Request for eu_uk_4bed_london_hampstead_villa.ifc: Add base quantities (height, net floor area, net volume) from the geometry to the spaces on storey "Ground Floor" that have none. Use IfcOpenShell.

First a look at what the model holds.

```python
import ifcopenshell
import ifcopenshell.util.element
import ifcopenshell.util.unit

model = ifcopenshell.open("eu_uk_4bed_london_hampstead_villa.ifc")
print(model.schema)
for unit_type in ("LENGTHUNIT", "AREAUNIT", "VOLUMEUNIT"):
    print(unit_type, ifcopenshell.util.unit.calculate_unit_scale(model, unit_type))
storey = next(s for s in model.by_type("IfcBuildingStorey") if s.Name == "Ground Floor")
spaces = [e for e in ifcopenshell.util.element.get_decomposition(storey) if e.is_a("IfcSpace")]
for e in sorted(spaces, key=lambda e: e.id()):
    print(e.id(), e.is_a(), e.Name, list(ifcopenshell.util.element.get_psets(e, qtos_only=True)), sep=" | ")
```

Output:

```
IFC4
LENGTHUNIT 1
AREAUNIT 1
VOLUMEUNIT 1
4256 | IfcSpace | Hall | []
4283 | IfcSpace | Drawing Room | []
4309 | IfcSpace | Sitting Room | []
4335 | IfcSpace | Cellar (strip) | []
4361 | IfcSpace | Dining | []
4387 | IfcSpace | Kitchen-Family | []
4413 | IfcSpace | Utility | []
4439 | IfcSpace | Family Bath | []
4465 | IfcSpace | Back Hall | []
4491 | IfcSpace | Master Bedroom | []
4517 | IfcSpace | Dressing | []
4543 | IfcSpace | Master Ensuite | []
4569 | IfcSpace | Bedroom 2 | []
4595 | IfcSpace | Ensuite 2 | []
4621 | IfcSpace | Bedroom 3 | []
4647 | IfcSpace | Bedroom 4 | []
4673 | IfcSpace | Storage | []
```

```python
import ifcopenshell
import ifcopenshell.api.pset
import ifcopenshell.geom
import ifcopenshell.util.element
import ifcopenshell.util.shape
import ifcopenshell.util.unit

model = ifcopenshell.open("eu_uk_4bed_london_hampstead_villa.ifc")
unit_scale = ifcopenshell.util.unit.calculate_unit_scale(model)
area_scale = ifcopenshell.util.unit.calculate_unit_scale(model, "AREAUNIT")
volume_scale = ifcopenshell.util.unit.calculate_unit_scale(model, "VOLUMEUNIT")
settings = ifcopenshell.geom.settings()

storey = next(s for s in model.by_type("IfcBuildingStorey") if s.Name == "Ground Floor")
spaces = [e for e in ifcopenshell.util.element.get_decomposition(storey) if e.is_a("IfcSpace")]

for e in sorted(spaces, key=lambda e: e.id()):
    if ifcopenshell.util.element.get_psets(e, qtos_only=True, should_inherit=False):
        continue
    # Geometry comes back in metres, in the element's own axes.
    shape = ifcopenshell.geom.create_shape(settings, e)
    values = {
        "Height": ifcopenshell.util.shape.get_z(shape.geometry) / unit_scale,
        "NetFloorArea": ifcopenshell.util.shape.get_footprint_area(shape.geometry) / area_scale,
        "NetVolume": ifcopenshell.util.shape.get_volume(shape.geometry) / volume_scale,
    }
    qto = ifcopenshell.api.pset.add_qto(model, product=e, name="Qto_SpaceBaseQuantities")
    ifcopenshell.api.pset.edit_qto(model, qto=qto, properties=values)
    print(e.id(), {k: round(v, 3) for k, v in values.items()})

model.write("eu_uk_4bed_london_hampstead_villa_updated.ifc")
```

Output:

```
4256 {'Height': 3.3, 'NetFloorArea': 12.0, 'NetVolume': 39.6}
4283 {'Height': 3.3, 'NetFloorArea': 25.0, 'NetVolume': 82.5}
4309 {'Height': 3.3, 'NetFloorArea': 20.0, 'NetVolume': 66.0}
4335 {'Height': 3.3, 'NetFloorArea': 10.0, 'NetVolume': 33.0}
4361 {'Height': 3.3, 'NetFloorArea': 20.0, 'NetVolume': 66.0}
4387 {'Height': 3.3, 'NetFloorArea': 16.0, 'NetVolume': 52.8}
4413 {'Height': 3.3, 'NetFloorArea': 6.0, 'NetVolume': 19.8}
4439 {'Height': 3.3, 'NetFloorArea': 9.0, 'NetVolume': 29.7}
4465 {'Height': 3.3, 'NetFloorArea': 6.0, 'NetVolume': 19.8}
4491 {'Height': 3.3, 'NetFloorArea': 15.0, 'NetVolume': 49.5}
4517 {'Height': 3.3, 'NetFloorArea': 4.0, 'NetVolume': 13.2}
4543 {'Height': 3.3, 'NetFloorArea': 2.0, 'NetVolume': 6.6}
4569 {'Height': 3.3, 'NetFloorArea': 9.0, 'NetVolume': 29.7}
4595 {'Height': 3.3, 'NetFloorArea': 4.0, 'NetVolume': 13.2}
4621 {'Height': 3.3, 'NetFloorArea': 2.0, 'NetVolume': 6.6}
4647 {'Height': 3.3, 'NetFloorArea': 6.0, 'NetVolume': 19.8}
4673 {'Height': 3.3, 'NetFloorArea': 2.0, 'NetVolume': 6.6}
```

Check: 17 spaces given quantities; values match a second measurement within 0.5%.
